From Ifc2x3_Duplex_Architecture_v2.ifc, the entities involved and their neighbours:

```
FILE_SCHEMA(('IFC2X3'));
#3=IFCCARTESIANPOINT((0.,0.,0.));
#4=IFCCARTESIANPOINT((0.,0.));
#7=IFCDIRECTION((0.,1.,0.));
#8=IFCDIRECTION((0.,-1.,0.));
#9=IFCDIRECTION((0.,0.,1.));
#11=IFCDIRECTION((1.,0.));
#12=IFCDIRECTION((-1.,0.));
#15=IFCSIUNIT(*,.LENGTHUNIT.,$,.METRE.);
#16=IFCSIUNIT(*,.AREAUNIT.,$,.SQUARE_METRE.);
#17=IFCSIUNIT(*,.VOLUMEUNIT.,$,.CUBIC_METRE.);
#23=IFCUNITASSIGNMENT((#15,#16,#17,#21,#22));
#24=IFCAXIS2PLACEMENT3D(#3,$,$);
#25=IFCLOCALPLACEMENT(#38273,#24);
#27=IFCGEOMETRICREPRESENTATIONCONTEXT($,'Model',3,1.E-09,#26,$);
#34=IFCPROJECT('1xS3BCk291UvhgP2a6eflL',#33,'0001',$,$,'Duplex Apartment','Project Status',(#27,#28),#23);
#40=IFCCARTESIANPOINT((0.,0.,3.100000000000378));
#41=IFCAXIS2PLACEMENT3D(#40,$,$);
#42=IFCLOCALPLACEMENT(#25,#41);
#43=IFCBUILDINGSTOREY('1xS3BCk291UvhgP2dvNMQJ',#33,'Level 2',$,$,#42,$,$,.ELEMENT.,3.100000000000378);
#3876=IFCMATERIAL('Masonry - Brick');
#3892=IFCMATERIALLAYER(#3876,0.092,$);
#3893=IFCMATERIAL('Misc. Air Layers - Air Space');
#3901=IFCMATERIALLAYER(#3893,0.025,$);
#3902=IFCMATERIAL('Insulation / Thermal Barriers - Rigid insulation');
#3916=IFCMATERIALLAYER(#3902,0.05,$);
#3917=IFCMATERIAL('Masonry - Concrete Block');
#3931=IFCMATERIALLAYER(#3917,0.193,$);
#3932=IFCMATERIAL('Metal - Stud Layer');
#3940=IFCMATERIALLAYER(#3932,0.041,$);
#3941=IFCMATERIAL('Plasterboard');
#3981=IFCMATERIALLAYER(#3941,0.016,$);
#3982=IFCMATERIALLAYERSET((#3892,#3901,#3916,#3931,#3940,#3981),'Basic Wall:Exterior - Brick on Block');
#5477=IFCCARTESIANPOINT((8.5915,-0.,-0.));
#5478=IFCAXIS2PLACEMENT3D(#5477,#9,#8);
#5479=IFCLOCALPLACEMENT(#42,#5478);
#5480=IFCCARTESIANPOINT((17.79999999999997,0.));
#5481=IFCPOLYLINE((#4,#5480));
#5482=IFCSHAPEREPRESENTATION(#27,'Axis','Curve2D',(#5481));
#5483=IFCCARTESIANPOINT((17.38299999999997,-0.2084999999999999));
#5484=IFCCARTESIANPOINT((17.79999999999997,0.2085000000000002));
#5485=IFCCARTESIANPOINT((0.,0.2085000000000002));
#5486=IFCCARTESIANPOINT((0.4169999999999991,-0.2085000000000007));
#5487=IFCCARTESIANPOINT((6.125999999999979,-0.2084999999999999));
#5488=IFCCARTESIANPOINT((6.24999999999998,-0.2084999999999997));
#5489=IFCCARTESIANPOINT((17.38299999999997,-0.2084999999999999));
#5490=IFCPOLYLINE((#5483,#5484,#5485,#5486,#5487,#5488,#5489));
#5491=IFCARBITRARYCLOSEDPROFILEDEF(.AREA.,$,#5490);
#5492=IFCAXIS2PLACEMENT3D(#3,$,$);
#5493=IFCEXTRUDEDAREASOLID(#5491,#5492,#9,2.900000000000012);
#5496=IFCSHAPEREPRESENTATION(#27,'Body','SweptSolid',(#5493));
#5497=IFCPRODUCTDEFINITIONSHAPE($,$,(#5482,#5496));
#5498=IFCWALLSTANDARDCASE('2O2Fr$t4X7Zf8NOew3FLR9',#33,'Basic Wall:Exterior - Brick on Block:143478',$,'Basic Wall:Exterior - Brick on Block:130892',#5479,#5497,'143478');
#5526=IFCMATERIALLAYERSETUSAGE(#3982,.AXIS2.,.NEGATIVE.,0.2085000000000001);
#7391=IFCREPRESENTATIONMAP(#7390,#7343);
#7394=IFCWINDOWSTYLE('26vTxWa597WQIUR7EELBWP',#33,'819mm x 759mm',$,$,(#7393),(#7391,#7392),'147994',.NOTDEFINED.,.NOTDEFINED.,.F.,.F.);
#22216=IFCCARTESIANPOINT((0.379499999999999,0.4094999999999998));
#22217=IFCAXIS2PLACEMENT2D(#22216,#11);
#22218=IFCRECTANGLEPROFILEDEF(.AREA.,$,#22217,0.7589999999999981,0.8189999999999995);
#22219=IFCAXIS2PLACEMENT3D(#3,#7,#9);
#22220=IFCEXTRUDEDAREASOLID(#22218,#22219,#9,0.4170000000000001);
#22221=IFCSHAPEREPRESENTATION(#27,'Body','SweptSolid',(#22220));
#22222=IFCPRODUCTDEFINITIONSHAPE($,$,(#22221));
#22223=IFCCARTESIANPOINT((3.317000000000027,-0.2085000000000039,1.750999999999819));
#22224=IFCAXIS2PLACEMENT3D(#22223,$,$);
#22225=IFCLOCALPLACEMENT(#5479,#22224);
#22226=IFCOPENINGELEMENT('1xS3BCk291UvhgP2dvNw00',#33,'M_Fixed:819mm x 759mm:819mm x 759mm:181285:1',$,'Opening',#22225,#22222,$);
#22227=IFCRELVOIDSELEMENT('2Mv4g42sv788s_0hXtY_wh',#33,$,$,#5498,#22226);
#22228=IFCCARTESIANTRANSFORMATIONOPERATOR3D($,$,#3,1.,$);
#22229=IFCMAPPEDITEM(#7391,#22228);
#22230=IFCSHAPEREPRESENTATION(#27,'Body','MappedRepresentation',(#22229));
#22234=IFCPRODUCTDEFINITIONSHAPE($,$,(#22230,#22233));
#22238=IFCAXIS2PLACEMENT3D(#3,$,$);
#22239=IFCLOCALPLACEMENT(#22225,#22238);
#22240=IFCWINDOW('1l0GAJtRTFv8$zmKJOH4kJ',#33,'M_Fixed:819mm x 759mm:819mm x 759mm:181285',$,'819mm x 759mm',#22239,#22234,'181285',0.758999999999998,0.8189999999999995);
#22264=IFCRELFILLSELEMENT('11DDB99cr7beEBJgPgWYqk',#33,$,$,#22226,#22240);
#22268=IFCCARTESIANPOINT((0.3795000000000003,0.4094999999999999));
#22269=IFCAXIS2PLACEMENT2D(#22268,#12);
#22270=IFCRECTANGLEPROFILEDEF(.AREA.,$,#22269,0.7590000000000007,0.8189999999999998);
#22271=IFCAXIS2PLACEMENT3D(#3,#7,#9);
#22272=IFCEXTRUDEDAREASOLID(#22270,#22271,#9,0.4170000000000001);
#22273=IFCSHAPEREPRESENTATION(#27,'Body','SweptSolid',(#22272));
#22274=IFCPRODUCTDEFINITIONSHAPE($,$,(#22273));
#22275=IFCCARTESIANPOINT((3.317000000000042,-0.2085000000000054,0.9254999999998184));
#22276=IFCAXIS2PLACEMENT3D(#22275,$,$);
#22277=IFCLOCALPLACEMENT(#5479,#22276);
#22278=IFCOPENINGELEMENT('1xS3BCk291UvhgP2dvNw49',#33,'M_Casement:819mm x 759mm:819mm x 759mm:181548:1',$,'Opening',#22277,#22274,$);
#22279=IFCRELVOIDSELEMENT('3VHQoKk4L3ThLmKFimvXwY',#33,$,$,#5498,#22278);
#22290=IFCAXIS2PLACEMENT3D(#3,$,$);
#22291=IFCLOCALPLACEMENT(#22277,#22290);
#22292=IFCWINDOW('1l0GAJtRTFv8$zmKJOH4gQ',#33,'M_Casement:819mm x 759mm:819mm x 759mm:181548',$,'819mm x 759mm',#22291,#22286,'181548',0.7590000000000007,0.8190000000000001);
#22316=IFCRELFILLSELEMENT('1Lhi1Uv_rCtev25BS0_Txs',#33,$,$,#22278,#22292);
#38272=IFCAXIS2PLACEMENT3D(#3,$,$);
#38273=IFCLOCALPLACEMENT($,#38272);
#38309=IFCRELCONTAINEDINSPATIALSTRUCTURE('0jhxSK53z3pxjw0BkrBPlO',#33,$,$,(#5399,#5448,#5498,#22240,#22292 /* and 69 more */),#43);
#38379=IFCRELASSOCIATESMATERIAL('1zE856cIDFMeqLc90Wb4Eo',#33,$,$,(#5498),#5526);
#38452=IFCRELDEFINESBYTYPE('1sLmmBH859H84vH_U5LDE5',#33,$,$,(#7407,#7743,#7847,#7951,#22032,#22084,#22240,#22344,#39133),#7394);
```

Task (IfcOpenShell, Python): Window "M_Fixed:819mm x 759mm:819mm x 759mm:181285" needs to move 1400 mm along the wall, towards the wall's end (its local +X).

```python
import ifcopenshell
import ifcopenshell.api.geometry
import ifcopenshell.util.placement

model = ifcopenshell.open("Ifc2x3_Duplex_Architecture_v2.ifc")

window = model.by_guid("1l0GAJtRTFv8$zmKJOH4kJ")
opening = window.FillsVoids[0].RelatingOpeningElement
wall = opening.VoidsElements[0].RelatingBuildingElement

wall_matrix = ifcopenshell.util.placement.get_local_placement(wall.ObjectPlacement)
shift = wall_matrix[:3, 0] * 1.4
before = ifcopenshell.util.placement.get_local_placement(window.ObjectPlacement)[:3, 3].copy()

# The window is placed relative to its opening, so it follows when the opening moves.
matrix = ifcopenshell.util.placement.get_local_placement(opening.ObjectPlacement)
matrix[:3, 3] += shift
ifcopenshell.api.geometry.edit_object_placement(
    model, product=opening, matrix=matrix, is_si=False, should_transform_children=True
)

after = ifcopenshell.util.placement.get_local_placement(window.ObjectPlacement)[:3, 3]
print("window moved by", (after - before).round(3) + 0.0)

model.write("Ifc2x3_Duplex_Architecture_v2-out.ifc")
```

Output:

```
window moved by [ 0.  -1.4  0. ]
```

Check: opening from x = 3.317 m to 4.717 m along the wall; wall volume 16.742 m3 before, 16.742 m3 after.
